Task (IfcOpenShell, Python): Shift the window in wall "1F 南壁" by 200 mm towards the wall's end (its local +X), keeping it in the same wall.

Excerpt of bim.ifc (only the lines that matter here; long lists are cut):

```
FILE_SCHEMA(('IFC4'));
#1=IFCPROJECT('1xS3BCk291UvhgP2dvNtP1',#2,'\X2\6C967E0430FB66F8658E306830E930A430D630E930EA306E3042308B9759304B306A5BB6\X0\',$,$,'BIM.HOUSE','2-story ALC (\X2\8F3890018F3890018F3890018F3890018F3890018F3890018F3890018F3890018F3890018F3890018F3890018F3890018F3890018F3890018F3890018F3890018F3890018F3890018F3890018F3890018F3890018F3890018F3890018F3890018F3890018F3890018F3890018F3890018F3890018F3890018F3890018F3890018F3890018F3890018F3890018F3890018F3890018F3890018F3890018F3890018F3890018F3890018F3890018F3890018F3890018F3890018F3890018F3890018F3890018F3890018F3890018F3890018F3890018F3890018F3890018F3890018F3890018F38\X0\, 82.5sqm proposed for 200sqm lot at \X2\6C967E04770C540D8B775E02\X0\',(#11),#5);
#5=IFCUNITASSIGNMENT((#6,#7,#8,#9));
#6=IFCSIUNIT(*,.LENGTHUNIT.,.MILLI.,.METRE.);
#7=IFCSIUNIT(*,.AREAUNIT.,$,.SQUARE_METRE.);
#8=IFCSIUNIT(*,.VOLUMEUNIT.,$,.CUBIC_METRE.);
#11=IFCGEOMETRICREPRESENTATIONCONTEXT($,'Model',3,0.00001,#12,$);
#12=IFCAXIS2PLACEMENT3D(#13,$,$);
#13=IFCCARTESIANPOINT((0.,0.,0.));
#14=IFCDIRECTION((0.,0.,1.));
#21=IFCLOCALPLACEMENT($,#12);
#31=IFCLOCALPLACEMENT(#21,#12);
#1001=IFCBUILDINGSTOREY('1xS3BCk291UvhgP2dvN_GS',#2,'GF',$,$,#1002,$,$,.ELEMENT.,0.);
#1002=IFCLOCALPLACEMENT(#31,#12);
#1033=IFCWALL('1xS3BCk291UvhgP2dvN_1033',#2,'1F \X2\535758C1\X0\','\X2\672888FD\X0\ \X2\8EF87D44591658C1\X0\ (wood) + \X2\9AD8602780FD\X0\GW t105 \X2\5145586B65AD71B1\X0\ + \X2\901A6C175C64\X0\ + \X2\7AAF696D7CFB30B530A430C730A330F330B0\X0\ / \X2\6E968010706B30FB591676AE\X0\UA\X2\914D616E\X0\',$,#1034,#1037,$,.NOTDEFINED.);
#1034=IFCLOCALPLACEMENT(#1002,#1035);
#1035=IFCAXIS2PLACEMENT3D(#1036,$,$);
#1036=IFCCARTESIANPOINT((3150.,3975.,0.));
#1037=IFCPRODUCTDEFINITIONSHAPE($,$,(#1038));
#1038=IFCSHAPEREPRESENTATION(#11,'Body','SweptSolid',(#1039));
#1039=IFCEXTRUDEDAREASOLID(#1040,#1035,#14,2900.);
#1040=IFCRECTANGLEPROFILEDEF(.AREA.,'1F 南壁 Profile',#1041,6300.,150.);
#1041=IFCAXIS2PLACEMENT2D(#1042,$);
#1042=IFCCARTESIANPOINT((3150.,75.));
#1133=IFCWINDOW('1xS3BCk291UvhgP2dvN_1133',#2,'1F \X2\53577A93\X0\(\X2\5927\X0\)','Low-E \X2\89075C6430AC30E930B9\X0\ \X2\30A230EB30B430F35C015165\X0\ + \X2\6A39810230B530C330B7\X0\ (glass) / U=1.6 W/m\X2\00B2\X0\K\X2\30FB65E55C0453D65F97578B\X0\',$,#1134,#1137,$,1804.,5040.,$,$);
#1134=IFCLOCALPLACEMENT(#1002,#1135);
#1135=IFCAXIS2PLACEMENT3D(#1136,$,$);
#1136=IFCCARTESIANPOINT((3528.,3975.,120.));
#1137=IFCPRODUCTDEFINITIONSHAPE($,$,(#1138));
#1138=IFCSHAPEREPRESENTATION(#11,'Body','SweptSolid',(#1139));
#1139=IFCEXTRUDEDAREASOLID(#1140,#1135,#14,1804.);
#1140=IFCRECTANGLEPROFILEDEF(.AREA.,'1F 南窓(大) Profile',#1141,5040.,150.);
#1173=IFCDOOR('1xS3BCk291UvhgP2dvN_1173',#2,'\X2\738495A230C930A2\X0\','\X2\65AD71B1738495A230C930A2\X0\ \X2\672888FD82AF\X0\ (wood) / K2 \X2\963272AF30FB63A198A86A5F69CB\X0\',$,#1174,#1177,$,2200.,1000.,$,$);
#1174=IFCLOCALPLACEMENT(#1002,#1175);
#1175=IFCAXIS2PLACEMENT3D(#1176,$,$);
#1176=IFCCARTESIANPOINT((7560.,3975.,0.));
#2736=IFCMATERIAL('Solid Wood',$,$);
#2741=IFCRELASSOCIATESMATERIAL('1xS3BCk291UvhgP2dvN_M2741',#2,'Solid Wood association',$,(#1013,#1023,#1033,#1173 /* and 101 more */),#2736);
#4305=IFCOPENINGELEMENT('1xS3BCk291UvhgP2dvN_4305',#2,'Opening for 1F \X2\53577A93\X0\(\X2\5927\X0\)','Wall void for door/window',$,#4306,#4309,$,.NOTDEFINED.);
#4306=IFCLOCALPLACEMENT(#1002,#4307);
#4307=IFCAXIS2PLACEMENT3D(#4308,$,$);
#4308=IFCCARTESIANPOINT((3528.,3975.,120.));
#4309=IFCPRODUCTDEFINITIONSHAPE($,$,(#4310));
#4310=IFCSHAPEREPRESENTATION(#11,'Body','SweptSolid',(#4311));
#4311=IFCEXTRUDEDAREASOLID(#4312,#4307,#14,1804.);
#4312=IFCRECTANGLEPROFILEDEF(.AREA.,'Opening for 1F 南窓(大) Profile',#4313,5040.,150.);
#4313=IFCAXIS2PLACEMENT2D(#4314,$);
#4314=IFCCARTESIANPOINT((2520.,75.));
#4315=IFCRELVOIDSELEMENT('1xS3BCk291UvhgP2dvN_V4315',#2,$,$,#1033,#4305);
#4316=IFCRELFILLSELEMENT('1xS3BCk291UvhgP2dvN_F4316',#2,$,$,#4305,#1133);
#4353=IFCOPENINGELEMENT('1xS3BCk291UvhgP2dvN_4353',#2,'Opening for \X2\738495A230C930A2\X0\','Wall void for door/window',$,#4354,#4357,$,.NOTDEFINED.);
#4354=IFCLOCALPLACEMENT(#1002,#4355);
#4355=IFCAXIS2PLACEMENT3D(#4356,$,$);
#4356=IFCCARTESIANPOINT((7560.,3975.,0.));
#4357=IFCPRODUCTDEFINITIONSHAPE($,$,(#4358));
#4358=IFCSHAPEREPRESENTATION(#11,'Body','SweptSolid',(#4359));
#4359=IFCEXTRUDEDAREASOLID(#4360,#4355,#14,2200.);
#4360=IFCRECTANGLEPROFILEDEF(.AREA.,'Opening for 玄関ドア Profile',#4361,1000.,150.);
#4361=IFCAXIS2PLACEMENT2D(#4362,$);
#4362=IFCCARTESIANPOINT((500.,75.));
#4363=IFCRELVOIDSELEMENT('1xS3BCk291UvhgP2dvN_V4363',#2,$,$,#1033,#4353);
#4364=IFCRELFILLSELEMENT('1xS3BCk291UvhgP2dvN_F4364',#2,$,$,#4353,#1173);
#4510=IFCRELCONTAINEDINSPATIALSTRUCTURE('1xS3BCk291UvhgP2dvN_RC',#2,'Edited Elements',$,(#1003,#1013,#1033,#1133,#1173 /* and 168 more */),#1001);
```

```python
import ifcopenshell
import ifcopenshell.api.geometry
import ifcopenshell.util.placement

model = ifcopenshell.open("bim.ifc")

window = model.by_id(1133)
opening = window.FillsVoids[0].RelatingOpeningElement
wall = opening.VoidsElements[0].RelatingBuildingElement

wall_matrix = ifcopenshell.util.placement.get_local_placement(wall.ObjectPlacement)
shift = wall_matrix[:3, 0] * 200.0
before = ifcopenshell.util.placement.get_local_placement(window.ObjectPlacement)[:3, 3].copy()

# The window is not placed relative to its opening, so move both.
for product in (opening, window):
    matrix = ifcopenshell.util.placement.get_local_placement(product.ObjectPlacement)
    matrix[:3, 3] += shift
    ifcopenshell.api.geometry.edit_object_placement(model, product=product, matrix=matrix, is_si=False)

after = ifcopenshell.util.placement.get_local_placement(window.ObjectPlacement)[:3, 3]
print("window moved by", (after - before).round(3) + 0.0)

model.write("bim-out.ifc")
```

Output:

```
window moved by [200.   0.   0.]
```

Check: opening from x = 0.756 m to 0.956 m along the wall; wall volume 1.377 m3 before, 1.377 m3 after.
